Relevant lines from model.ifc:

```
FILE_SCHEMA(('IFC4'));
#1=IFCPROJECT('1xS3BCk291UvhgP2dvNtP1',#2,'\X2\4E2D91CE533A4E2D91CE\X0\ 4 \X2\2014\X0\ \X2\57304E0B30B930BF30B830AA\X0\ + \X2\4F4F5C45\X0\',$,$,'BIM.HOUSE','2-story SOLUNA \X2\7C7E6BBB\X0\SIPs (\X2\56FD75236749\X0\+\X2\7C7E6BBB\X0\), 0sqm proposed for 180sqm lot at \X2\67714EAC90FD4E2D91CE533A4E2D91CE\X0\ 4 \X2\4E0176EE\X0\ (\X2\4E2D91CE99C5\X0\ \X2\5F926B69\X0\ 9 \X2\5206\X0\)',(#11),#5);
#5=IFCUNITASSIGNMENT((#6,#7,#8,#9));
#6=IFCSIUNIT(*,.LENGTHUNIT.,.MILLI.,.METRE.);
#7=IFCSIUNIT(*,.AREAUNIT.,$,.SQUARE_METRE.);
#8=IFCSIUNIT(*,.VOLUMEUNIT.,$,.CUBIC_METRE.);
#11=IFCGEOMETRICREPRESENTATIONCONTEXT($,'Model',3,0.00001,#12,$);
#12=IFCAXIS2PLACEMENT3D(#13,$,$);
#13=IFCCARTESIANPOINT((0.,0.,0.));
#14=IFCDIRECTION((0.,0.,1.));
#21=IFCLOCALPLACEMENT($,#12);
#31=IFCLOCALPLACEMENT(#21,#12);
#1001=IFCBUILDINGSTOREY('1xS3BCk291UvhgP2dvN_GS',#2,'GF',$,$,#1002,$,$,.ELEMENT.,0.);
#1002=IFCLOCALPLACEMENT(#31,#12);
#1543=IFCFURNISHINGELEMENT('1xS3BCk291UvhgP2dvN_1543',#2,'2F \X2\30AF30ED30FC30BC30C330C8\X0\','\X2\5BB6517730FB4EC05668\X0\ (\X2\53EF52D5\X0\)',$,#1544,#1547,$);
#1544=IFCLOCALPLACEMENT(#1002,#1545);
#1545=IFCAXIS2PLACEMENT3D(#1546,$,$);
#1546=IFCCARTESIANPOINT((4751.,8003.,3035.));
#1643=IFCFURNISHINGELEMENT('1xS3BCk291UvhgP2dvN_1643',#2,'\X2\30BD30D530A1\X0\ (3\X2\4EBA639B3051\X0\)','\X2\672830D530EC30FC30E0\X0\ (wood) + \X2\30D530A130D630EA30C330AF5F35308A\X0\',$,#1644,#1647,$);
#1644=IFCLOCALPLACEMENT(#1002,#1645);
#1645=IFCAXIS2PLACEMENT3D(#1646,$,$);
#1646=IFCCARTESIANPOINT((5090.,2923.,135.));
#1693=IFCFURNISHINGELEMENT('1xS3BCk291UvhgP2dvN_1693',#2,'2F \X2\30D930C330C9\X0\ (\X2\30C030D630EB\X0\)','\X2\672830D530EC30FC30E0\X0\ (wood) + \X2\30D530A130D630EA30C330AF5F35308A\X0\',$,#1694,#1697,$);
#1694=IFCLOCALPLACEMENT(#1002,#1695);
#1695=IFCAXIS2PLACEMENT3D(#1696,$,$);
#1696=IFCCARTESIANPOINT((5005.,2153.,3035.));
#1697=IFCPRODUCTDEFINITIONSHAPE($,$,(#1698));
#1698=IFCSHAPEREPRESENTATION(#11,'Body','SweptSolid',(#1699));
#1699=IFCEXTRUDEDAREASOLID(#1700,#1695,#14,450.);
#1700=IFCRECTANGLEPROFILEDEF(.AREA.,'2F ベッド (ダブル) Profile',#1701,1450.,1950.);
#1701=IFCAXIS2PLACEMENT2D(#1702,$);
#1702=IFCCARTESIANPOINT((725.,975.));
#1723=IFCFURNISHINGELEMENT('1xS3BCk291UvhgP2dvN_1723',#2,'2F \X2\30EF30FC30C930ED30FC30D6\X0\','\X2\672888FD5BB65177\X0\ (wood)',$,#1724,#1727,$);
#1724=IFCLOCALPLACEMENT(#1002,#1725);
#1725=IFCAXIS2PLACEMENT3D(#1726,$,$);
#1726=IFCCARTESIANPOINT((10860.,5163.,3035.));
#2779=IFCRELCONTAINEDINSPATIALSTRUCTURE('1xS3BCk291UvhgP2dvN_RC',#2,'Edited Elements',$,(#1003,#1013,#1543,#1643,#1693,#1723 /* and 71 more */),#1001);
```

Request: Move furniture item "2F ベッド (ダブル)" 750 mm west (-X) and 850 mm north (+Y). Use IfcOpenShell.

```python
import ifcopenshell
import ifcopenshell.api.geometry
import ifcopenshell.util.placement
import ifcopenshell.util.unit

model = ifcopenshell.open("model.ifc")
unit_scale = ifcopenshell.util.unit.calculate_unit_scale(model)

item = model.by_guid("1xS3BCk291UvhgP2dvN_1693")
matrix = ifcopenshell.util.placement.get_local_placement(item.ObjectPlacement)
matrix[0, 3] -= 0.75 / unit_scale
matrix[1, 3] += 0.85 / unit_scale
ifcopenshell.api.geometry.edit_object_placement(model, product=item, matrix=matrix, is_si=False)

print(ifcopenshell.util.placement.get_local_placement(item.ObjectPlacement).round(3) + 0.0)

model.write("model_updated.ifc")
```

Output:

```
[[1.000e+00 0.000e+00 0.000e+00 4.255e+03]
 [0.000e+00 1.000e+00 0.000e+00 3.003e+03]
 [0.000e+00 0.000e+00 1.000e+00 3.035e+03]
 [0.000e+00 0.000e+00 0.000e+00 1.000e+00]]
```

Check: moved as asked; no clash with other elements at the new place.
